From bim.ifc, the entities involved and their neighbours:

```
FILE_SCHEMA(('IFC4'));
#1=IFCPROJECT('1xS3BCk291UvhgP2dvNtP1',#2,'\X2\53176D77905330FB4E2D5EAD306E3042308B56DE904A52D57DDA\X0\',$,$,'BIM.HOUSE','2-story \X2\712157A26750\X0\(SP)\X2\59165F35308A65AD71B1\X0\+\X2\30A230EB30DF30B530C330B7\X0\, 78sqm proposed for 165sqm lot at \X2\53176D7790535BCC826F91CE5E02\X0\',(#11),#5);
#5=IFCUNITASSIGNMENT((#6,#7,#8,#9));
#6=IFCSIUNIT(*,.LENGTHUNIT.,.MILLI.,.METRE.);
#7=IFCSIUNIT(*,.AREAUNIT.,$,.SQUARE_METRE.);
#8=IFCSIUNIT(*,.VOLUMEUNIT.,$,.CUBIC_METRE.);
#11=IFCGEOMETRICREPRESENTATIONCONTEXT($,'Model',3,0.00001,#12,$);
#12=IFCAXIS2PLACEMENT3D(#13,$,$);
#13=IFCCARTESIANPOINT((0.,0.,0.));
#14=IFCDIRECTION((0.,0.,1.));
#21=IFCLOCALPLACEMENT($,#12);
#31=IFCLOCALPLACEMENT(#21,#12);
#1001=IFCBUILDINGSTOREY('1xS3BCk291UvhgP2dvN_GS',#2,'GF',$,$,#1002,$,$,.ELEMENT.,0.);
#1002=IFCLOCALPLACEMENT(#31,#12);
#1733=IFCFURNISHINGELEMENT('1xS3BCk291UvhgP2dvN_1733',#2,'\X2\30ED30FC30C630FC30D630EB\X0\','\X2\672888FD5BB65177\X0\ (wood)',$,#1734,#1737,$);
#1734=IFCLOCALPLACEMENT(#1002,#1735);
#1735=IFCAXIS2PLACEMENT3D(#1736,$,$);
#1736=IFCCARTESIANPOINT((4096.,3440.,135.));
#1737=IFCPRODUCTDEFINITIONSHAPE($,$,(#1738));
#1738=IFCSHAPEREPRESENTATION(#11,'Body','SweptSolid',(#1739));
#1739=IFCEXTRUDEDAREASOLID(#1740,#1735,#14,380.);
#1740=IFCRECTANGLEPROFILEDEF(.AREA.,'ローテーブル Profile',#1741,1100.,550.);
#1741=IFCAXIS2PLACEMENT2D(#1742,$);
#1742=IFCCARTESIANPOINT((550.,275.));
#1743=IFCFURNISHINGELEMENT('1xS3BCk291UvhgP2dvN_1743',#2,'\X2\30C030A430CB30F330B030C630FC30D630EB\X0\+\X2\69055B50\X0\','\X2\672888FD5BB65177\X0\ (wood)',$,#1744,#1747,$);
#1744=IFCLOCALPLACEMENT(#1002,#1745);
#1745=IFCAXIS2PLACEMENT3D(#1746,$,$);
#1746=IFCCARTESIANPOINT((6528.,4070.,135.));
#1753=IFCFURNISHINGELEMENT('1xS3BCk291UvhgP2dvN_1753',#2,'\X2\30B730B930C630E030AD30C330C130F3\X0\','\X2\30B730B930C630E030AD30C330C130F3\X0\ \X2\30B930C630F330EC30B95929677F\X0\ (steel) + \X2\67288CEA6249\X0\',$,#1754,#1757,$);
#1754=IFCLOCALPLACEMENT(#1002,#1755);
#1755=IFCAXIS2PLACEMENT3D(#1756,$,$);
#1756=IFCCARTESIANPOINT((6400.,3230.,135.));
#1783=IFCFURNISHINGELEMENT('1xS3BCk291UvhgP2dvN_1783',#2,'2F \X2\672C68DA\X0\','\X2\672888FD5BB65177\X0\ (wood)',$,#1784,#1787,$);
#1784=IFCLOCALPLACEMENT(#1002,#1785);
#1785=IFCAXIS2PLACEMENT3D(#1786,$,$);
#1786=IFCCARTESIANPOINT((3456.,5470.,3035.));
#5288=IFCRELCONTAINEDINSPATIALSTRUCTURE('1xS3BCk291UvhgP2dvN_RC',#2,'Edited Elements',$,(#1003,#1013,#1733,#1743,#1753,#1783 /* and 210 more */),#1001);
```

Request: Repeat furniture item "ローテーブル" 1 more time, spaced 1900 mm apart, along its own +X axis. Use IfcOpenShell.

```python
import ifcopenshell
import ifcopenshell.api.geometry
import ifcopenshell.api.root
import ifcopenshell.util.element
import ifcopenshell.util.placement
import ifcopenshell.util.unit

model = ifcopenshell.open("bim.ifc")
unit_scale = ifcopenshell.util.unit.calculate_unit_scale(model)


def reuse_history(source, copy):
    """copy_class also copies each property set's owner history, people and application; keep the originals."""
    for rel in copy.IsDefinedBy:
        if rel.is_a("IfcRelDefinesByProperties") and (history := rel.RelatingPropertyDefinition.OwnerHistory):
            rel.RelatingPropertyDefinition.OwnerHistory = source.OwnerHistory
            ifcopenshell.util.element.remove_deep2(model, history)


source = model.by_guid("1xS3BCk291UvhgP2dvN_1733")
base = ifcopenshell.util.placement.get_local_placement(source.ObjectPlacement)
step = base[:3, 0] * 1.9 / unit_scale

for i in range(1, 2):
    copy = ifcopenshell.api.root.copy_class(model, product=source)
    copy.Representation = ifcopenshell.util.element.copy_deep(
        model, source.Representation, exclude=["IfcGeometricRepresentationContext", "IfcRepresentationMap"]
    )
    reuse_history(source, copy)
    matrix = base.copy()
    matrix[:3, 3] += i * step
    print("added at", matrix[:3, 3].round(3) + 0.0)
    ifcopenshell.api.geometry.edit_object_placement(model, product=copy, matrix=matrix, is_si=False)

model.write("bim_edited.ifc")
```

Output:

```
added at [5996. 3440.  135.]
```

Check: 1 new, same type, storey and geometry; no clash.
